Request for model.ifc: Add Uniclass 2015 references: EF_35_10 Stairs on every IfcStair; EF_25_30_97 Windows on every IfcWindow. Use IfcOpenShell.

First a look at what the model holds.

```python
import ifcopenshell

model = ifcopenshell.open("model.ifc")
print(model.schema)
print("classifications:", [c.Name for c in model.by_type("IfcClassification")])
for ifc_class in ("IfcDoor", "IfcRoof", "IfcStair", "IfcWall", "IfcWindow"):
    print(ifc_class, len(model.by_type(ifc_class)))
```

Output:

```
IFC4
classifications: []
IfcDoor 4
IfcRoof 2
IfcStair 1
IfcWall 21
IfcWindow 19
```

```python
import ifcopenshell
import ifcopenshell.api.classification

model = ifcopenshell.open("model.ifc")

system = ifcopenshell.api.classification.add_classification(model, classification="Uniclass 2015")

codes = {
    "IfcStair": ("EF_35_10", "Stairs"),
    "IfcWindow": ("EF_25_30_97", "Windows"),
}
for ifc_class, (code, name) in codes.items():
    products = model.by_type(ifc_class)
    ifcopenshell.api.classification.add_reference(
        model, products=products, classification=system, identification=code, name=name
    )
    print(code, len(products))

model.write("model-out.ifc")
```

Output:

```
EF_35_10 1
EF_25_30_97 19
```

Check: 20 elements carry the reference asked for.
